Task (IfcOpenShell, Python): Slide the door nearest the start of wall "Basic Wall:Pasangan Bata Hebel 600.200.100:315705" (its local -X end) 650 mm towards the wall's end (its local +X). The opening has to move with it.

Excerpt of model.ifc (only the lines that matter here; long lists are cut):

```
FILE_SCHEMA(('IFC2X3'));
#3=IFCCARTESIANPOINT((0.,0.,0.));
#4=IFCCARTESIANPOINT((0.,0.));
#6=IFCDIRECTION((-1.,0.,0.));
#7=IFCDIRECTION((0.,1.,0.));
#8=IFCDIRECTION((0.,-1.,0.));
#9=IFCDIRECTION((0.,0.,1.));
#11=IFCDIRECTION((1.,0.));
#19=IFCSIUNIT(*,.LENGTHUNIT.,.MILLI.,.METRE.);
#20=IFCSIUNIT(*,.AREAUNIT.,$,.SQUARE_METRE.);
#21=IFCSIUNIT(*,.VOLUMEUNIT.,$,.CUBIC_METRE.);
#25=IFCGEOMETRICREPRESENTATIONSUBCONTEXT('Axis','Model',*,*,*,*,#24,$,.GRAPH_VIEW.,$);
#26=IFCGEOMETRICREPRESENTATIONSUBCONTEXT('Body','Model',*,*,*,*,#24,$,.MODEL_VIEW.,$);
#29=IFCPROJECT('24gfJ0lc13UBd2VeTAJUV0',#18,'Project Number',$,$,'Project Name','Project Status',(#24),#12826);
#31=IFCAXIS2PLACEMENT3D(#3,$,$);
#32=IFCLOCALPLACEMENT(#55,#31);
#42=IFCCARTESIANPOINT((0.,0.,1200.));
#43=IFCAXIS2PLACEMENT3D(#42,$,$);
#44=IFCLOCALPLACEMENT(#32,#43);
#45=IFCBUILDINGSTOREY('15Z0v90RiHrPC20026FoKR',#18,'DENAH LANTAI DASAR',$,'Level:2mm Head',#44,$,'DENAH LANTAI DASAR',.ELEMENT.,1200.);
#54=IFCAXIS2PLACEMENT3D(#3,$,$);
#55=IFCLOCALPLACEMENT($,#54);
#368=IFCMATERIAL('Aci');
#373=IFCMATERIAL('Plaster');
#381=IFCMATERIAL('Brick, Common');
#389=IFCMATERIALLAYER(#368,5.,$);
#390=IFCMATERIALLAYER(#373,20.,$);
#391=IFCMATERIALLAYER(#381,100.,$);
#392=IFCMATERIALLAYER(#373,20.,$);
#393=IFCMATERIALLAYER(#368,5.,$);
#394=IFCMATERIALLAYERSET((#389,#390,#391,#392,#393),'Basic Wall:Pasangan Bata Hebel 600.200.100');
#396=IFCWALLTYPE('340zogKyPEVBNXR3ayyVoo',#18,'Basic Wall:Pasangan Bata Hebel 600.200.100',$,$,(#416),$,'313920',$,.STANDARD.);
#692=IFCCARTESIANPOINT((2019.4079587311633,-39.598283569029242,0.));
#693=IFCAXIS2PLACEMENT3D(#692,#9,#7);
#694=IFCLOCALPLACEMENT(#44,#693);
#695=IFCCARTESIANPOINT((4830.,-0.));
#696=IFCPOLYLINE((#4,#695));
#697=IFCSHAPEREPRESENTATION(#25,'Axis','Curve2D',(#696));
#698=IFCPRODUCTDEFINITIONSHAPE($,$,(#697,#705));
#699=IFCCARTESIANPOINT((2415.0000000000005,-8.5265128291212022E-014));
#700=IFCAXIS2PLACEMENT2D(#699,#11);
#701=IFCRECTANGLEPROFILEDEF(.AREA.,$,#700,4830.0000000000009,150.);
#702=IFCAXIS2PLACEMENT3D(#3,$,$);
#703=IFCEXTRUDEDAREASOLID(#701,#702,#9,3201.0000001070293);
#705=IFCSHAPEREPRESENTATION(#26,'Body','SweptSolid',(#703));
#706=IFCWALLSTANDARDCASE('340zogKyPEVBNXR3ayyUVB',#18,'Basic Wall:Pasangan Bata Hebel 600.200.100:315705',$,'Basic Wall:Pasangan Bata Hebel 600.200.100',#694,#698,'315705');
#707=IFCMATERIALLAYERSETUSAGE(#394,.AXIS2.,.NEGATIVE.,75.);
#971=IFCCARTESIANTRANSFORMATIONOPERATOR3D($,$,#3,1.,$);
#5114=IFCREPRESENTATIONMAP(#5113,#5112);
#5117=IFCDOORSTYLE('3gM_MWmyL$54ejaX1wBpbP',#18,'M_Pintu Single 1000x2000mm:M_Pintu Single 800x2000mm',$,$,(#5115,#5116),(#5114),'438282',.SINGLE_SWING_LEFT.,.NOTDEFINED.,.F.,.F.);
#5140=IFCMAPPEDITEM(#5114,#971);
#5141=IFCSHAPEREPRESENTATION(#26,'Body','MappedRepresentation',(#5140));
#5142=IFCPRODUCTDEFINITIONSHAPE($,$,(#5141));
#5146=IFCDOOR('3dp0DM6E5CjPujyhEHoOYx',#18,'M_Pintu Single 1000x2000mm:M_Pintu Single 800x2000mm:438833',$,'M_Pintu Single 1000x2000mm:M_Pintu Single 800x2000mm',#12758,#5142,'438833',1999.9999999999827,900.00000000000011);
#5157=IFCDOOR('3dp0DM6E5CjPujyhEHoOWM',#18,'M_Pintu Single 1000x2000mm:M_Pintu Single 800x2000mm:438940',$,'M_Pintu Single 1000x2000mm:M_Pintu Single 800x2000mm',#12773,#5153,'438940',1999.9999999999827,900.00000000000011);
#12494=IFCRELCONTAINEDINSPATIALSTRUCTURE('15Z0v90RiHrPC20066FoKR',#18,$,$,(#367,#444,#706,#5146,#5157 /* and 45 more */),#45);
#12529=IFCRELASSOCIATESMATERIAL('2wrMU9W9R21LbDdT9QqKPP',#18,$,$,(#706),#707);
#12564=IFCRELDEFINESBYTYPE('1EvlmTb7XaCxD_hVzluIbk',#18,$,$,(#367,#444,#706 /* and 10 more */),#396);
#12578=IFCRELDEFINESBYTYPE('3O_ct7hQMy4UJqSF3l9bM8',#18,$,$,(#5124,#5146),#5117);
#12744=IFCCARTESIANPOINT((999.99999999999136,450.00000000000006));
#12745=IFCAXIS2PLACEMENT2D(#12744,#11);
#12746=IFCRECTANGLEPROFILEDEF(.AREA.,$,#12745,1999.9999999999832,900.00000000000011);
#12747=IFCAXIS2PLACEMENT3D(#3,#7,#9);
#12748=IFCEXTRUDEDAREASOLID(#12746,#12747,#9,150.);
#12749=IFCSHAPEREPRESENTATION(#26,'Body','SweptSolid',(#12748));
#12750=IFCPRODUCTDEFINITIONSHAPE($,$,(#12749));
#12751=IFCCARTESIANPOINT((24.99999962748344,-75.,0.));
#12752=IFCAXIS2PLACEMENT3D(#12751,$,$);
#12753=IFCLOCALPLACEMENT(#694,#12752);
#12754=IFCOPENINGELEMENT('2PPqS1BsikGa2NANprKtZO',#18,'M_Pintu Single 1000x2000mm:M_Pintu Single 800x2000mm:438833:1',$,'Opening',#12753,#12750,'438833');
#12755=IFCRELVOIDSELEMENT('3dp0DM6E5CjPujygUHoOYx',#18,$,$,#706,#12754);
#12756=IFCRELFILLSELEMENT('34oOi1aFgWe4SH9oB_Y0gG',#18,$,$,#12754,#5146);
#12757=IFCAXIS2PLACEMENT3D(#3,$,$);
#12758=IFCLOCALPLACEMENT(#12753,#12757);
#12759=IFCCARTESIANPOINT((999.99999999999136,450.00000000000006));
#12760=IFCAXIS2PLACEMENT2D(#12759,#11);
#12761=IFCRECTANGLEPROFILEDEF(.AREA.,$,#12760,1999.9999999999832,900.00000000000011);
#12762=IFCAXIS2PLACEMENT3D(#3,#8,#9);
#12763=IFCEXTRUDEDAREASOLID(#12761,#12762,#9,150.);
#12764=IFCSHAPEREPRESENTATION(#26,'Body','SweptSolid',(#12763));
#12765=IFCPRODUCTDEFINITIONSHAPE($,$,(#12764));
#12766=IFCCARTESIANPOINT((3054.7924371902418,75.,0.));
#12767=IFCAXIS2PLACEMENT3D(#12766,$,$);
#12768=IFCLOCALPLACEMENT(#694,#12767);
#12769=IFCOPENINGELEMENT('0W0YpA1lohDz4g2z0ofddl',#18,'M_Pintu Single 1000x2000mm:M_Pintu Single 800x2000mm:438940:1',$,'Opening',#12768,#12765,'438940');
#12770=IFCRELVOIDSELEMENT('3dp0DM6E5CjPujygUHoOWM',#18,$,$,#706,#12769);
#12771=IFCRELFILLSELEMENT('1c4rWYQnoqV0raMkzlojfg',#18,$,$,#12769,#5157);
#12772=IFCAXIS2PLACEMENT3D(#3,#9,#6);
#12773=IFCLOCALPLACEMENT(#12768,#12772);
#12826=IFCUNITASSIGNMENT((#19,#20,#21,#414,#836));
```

```python
import ifcopenshell
import ifcopenshell.api.geometry
import ifcopenshell.util.placement

model = ifcopenshell.open("model.ifc")

door = model.by_guid("3dp0DM6E5CjPujyhEHoOYx")
opening = door.FillsVoids[0].RelatingOpeningElement
wall = opening.VoidsElements[0].RelatingBuildingElement

wall_matrix = ifcopenshell.util.placement.get_local_placement(wall.ObjectPlacement)
shift = wall_matrix[:3, 0] * 650.0
before = ifcopenshell.util.placement.get_local_placement(door.ObjectPlacement)[:3, 3].copy()

# The door is placed relative to its opening, so it follows when the opening moves.
matrix = ifcopenshell.util.placement.get_local_placement(opening.ObjectPlacement)
matrix[:3, 3] += shift
ifcopenshell.api.geometry.edit_object_placement(
    model, product=opening, matrix=matrix, is_si=False, should_transform_children=True
)

after = ifcopenshell.util.placement.get_local_placement(door.ObjectPlacement)[:3, 3]
print("door moved by", (after - before).round(3) + 0.0)

model.write("model_updated.ifc")
```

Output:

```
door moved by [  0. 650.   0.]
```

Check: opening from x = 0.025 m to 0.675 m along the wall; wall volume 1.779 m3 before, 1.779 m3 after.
